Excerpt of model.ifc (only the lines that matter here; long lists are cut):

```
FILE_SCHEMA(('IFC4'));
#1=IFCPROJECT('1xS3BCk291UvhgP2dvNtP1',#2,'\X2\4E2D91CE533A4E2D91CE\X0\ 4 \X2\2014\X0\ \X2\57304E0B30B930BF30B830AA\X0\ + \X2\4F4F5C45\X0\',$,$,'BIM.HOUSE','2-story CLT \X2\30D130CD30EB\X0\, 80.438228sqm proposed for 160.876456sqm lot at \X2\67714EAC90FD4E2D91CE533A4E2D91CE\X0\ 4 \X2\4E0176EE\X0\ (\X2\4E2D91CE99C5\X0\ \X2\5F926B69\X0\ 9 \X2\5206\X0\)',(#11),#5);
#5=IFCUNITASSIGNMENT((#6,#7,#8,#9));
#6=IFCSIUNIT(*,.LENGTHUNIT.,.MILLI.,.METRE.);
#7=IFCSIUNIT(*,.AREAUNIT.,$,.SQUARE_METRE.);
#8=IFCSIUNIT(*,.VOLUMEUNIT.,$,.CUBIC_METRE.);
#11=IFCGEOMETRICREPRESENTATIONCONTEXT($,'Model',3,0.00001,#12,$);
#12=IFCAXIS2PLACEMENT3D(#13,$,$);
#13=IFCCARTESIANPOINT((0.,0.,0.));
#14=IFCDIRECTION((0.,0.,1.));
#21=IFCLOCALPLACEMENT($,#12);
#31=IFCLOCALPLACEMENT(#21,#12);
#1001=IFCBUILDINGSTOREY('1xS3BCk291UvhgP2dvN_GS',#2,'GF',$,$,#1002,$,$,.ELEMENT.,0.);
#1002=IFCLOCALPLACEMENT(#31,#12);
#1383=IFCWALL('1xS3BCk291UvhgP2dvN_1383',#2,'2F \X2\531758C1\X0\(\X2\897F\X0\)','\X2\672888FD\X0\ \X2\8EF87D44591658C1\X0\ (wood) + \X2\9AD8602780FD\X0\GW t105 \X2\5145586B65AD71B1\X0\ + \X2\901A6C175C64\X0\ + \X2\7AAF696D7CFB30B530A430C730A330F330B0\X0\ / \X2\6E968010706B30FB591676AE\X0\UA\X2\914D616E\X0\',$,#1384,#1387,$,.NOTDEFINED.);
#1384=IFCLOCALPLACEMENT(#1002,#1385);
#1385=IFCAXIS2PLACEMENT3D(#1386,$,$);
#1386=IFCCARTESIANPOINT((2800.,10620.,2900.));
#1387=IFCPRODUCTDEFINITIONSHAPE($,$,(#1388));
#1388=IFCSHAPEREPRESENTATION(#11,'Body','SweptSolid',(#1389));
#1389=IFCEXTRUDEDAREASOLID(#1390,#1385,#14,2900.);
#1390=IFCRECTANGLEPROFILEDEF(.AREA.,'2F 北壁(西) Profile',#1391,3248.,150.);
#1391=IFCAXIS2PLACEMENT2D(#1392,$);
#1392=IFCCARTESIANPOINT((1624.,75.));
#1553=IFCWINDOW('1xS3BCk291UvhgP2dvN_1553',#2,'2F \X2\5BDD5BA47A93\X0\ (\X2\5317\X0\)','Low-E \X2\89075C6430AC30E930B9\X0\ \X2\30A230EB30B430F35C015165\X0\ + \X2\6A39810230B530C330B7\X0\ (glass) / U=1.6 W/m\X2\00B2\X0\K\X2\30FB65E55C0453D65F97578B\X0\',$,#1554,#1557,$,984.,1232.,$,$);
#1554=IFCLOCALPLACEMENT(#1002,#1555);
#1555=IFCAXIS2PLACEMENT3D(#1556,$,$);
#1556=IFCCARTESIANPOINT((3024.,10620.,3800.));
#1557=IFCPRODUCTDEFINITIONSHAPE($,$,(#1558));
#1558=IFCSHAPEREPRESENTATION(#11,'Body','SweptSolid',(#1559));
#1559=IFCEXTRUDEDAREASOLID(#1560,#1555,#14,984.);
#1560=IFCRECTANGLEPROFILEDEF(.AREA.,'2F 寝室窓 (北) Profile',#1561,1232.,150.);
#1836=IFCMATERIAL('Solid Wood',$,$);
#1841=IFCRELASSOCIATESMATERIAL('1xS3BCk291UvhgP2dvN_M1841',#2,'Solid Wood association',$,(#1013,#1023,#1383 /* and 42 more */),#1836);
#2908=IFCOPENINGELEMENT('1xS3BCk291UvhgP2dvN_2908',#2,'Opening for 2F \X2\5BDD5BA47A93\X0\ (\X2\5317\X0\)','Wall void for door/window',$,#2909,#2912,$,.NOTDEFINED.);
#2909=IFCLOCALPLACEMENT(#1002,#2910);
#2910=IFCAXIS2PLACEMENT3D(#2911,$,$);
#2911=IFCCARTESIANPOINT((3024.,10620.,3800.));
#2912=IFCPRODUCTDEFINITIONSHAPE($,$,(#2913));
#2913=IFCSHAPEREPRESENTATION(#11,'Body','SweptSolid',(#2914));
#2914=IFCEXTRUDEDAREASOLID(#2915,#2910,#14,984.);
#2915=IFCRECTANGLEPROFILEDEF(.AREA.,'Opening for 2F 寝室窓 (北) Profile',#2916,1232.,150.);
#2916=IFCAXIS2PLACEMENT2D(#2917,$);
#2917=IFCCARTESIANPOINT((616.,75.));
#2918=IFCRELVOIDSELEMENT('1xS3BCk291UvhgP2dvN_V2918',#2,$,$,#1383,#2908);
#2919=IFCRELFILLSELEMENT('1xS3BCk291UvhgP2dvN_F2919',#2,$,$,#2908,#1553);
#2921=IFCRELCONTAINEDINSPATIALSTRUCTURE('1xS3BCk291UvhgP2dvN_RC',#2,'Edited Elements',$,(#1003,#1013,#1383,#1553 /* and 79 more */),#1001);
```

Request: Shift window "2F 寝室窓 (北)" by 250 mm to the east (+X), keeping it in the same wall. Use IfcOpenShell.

```python
import ifcopenshell
import ifcopenshell.api.geometry
import ifcopenshell.util.placement

model = ifcopenshell.open("model.ifc")

window = model.by_guid("1xS3BCk291UvhgP2dvN_1553")
opening = window.FillsVoids[0].RelatingOpeningElement
wall = opening.VoidsElements[0].RelatingBuildingElement

wall_matrix = ifcopenshell.util.placement.get_local_placement(wall.ObjectPlacement)
shift = wall_matrix[:3, 0] * 250.0
before = ifcopenshell.util.placement.get_local_placement(window.ObjectPlacement)[:3, 3].copy()

# The window is not placed relative to its opening, so move both.
for product in (opening, window):
    matrix = ifcopenshell.util.placement.get_local_placement(product.ObjectPlacement)
    matrix[:3, 3] += shift
    ifcopenshell.api.geometry.edit_object_placement(model, product=product, matrix=matrix, is_si=False)

after = ifcopenshell.util.placement.get_local_placement(window.ObjectPlacement)[:3, 3]
print("window moved by", (after - before).round(3) + 0.0)

model.write("model_updated.ifc")
```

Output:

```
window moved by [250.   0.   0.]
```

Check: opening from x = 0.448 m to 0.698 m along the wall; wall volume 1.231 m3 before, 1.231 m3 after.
